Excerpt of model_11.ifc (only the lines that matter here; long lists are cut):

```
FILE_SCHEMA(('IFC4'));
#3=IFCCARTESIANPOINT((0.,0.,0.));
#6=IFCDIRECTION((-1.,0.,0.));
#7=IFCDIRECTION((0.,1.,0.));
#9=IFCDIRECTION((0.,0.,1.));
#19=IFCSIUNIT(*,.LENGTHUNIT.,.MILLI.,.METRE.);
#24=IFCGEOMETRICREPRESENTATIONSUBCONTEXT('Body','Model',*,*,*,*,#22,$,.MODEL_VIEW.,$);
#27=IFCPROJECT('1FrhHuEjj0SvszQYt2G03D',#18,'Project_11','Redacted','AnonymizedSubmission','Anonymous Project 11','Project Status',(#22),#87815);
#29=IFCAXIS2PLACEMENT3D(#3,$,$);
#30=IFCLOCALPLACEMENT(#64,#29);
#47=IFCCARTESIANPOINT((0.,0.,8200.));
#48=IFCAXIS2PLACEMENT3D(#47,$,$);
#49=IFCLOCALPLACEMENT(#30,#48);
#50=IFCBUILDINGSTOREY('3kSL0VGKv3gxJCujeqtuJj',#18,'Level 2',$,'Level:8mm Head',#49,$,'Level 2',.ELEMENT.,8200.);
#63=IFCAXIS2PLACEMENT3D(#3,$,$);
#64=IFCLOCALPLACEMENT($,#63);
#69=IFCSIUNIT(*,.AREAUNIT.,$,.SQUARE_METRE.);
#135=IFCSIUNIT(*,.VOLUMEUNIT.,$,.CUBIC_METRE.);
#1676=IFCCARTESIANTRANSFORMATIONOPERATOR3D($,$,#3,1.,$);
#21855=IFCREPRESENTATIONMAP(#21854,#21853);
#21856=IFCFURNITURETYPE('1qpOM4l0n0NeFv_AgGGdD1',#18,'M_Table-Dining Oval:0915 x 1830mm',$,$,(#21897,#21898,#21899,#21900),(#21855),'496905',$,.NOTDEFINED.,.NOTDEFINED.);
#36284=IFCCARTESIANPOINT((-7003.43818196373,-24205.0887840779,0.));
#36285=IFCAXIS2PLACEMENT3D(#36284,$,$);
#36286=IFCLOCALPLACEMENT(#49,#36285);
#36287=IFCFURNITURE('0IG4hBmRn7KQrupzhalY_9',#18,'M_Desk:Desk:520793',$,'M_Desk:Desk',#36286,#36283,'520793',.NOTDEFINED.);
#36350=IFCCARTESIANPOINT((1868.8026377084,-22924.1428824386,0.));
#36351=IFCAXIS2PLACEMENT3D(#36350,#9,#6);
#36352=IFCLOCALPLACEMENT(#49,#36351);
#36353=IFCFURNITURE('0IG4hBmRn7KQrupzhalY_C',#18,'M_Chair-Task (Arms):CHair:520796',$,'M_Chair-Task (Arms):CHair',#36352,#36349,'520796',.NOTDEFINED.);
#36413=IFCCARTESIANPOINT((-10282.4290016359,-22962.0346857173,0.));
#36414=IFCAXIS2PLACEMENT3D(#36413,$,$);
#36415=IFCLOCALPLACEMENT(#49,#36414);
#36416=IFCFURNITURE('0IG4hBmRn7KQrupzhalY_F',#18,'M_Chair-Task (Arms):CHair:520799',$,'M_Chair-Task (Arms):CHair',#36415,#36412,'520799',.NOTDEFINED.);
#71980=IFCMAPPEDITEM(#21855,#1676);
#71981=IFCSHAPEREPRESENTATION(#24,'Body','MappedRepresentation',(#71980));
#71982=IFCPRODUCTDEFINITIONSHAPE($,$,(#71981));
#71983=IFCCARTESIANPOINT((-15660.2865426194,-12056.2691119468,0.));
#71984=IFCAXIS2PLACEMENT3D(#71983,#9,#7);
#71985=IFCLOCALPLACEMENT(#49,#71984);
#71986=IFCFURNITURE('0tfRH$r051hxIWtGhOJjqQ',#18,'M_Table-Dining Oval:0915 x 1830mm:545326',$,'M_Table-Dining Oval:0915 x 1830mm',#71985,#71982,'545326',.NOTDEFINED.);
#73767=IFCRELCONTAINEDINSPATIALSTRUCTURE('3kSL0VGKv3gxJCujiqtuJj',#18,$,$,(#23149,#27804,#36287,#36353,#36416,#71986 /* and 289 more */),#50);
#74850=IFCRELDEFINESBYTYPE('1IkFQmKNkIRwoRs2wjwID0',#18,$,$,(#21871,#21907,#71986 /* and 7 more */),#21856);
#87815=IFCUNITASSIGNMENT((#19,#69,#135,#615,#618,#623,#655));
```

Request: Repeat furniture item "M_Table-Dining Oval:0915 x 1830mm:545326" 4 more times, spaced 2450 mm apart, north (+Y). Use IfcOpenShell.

```python
import numpy as np
import ifcopenshell
import ifcopenshell.api.geometry
import ifcopenshell.api.root
import ifcopenshell.util.element
import ifcopenshell.util.placement
import ifcopenshell.util.unit

model = ifcopenshell.open("model_11.ifc")
unit_scale = ifcopenshell.util.unit.calculate_unit_scale(model)


def reuse_history(source, copy):
    """copy_class also copies each property set's owner history, people and application; keep the originals."""
    for rel in copy.IsDefinedBy:
        if rel.is_a("IfcRelDefinesByProperties") and (history := rel.RelatingPropertyDefinition.OwnerHistory):
            rel.RelatingPropertyDefinition.OwnerHistory = source.OwnerHistory
            ifcopenshell.util.element.remove_deep2(model, history)


source = model.by_id(71986)
base = ifcopenshell.util.placement.get_local_placement(source.ObjectPlacement)
step = np.array([0.0, 1.0, 0.0]) * 2.45 / unit_scale

for i in range(1, 5):
    copy = ifcopenshell.api.root.copy_class(model, product=source)
    copy.Representation = ifcopenshell.util.element.copy_deep(
        model, source.Representation, exclude=["IfcGeometricRepresentationContext", "IfcRepresentationMap"]
    )
    copy.Name = "M_Table-Dining Oval:0915 x 1830mm"
    copy.Tag = None
    reuse_history(source, copy)
    matrix = base.copy()
    matrix[:3, 3] += i * step
    print("added at", matrix[:3, 3].round(3) + 0.0)
    ifcopenshell.api.geometry.edit_object_placement(model, product=copy, matrix=matrix, is_si=False)

model.write("model_11-out.ifc")
```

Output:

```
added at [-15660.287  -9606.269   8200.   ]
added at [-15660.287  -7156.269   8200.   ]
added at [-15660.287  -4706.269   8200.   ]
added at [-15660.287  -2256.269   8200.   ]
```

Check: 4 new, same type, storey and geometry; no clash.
